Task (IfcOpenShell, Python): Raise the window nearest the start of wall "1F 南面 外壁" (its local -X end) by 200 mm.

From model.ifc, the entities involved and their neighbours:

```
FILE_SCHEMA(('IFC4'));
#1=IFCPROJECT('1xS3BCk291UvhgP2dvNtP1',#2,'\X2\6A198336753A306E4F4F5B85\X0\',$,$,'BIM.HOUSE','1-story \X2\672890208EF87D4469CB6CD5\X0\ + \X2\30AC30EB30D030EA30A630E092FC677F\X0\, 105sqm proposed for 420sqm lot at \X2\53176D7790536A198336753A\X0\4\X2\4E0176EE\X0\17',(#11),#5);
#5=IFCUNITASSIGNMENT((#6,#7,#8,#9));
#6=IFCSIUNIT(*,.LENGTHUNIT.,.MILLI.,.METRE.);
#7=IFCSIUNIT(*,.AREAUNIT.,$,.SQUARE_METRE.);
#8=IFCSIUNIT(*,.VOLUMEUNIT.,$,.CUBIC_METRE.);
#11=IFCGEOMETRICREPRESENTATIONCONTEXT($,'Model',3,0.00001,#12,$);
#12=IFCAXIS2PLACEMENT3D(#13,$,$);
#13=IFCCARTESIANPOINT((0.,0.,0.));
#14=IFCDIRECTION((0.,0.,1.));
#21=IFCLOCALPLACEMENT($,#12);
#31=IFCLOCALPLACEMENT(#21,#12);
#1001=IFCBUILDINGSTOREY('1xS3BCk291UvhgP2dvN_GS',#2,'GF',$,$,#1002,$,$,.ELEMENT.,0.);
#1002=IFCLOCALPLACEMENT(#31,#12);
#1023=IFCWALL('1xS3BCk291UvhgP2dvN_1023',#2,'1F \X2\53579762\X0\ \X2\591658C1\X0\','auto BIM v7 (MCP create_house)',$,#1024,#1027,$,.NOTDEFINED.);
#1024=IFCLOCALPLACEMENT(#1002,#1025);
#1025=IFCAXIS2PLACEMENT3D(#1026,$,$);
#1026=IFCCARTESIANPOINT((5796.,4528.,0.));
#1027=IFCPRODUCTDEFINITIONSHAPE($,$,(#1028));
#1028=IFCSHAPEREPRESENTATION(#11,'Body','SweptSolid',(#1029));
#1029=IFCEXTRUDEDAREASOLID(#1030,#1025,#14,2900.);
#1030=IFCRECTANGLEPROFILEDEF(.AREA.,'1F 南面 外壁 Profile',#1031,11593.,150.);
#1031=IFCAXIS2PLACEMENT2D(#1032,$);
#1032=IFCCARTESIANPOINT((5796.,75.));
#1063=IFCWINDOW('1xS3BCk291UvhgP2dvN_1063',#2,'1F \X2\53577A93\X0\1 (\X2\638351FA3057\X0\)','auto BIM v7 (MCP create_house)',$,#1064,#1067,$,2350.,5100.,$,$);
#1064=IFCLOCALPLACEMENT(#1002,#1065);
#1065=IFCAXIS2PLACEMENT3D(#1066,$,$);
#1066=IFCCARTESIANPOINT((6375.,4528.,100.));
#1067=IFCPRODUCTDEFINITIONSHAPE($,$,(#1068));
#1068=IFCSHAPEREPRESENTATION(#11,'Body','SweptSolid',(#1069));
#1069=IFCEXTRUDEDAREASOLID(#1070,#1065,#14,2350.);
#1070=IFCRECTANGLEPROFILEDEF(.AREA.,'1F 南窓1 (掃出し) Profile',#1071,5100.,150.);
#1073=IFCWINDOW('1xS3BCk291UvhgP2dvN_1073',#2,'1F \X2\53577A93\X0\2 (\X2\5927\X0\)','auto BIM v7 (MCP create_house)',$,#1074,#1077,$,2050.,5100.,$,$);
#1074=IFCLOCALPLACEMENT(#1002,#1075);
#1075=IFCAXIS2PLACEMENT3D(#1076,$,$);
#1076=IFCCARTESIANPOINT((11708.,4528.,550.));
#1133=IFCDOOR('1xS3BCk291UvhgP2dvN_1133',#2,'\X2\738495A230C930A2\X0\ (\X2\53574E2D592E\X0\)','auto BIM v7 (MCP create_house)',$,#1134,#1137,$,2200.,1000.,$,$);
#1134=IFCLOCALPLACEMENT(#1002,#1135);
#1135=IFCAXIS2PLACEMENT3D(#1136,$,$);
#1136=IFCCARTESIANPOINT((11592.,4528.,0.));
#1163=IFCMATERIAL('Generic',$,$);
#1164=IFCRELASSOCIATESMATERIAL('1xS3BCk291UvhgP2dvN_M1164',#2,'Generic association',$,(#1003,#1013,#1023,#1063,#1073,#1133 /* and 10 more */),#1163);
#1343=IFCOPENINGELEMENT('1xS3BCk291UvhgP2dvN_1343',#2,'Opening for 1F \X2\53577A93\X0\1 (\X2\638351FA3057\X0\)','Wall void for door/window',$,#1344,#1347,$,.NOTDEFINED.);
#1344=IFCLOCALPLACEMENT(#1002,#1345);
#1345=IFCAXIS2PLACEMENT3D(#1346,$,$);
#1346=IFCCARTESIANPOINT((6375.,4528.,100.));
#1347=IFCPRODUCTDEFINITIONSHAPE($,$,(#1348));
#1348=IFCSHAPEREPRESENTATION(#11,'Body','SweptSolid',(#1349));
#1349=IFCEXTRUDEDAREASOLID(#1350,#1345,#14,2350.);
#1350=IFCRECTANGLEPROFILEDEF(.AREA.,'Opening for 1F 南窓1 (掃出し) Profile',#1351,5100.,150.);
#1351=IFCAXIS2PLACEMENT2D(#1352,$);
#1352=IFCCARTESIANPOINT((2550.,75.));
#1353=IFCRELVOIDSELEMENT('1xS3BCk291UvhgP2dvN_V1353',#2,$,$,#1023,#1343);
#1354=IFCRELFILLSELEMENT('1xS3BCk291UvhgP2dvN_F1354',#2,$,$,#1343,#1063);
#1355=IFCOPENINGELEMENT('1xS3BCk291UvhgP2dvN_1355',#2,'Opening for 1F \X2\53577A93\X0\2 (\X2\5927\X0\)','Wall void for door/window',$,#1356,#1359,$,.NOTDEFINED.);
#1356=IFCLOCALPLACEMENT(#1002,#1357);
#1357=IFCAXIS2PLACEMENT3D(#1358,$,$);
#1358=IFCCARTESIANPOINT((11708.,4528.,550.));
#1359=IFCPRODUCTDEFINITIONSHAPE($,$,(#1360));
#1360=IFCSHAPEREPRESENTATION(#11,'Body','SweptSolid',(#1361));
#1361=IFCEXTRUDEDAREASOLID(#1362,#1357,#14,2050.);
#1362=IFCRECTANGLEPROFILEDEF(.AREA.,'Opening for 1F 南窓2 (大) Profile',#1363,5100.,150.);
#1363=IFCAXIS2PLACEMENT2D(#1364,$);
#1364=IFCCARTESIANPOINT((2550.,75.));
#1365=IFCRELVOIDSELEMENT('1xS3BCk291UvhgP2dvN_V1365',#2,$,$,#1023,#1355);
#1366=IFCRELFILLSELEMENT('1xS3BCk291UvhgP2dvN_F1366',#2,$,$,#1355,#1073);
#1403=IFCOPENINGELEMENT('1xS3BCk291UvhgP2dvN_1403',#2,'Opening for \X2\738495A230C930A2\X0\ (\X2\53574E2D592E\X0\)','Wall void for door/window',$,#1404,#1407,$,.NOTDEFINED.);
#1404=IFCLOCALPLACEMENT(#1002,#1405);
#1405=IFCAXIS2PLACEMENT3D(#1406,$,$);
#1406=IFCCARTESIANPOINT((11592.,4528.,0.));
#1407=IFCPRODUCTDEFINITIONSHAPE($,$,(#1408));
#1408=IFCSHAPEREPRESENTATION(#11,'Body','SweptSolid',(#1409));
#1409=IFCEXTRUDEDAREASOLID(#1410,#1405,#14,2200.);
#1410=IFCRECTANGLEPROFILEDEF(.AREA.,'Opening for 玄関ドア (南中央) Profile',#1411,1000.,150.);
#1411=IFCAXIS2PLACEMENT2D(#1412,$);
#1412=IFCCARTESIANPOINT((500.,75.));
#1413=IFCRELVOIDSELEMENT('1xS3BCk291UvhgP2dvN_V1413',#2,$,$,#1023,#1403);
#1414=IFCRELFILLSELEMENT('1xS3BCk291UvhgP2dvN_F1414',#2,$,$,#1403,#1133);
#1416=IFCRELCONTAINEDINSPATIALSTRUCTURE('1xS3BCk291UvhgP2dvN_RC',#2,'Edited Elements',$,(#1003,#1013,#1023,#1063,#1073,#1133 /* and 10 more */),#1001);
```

```python
import numpy as np
import ifcopenshell
import ifcopenshell.api.geometry
import ifcopenshell.util.placement
import ifcopenshell.util.unit

model = ifcopenshell.open("model.ifc")
unit_scale = ifcopenshell.util.unit.calculate_unit_scale(model)

window = model.by_guid("1xS3BCk291UvhgP2dvN_1063")
opening = window.FillsVoids[0].RelatingOpeningElement
dz = 200.0

shift = np.array([0.0, 0.0, dz])
# The window is not placed relative to its opening, so move both.
for product in (opening, window):
    matrix = ifcopenshell.util.placement.get_local_placement(product.ObjectPlacement)
    matrix[:3, 3] += shift
    ifcopenshell.api.geometry.edit_object_placement(model, product=product, matrix=matrix, is_si=False)

print(f"moved by {dz * unit_scale:+.3f} m")

model.write("model_v2.ifc")
```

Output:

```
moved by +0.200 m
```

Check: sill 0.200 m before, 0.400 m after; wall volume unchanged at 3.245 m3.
